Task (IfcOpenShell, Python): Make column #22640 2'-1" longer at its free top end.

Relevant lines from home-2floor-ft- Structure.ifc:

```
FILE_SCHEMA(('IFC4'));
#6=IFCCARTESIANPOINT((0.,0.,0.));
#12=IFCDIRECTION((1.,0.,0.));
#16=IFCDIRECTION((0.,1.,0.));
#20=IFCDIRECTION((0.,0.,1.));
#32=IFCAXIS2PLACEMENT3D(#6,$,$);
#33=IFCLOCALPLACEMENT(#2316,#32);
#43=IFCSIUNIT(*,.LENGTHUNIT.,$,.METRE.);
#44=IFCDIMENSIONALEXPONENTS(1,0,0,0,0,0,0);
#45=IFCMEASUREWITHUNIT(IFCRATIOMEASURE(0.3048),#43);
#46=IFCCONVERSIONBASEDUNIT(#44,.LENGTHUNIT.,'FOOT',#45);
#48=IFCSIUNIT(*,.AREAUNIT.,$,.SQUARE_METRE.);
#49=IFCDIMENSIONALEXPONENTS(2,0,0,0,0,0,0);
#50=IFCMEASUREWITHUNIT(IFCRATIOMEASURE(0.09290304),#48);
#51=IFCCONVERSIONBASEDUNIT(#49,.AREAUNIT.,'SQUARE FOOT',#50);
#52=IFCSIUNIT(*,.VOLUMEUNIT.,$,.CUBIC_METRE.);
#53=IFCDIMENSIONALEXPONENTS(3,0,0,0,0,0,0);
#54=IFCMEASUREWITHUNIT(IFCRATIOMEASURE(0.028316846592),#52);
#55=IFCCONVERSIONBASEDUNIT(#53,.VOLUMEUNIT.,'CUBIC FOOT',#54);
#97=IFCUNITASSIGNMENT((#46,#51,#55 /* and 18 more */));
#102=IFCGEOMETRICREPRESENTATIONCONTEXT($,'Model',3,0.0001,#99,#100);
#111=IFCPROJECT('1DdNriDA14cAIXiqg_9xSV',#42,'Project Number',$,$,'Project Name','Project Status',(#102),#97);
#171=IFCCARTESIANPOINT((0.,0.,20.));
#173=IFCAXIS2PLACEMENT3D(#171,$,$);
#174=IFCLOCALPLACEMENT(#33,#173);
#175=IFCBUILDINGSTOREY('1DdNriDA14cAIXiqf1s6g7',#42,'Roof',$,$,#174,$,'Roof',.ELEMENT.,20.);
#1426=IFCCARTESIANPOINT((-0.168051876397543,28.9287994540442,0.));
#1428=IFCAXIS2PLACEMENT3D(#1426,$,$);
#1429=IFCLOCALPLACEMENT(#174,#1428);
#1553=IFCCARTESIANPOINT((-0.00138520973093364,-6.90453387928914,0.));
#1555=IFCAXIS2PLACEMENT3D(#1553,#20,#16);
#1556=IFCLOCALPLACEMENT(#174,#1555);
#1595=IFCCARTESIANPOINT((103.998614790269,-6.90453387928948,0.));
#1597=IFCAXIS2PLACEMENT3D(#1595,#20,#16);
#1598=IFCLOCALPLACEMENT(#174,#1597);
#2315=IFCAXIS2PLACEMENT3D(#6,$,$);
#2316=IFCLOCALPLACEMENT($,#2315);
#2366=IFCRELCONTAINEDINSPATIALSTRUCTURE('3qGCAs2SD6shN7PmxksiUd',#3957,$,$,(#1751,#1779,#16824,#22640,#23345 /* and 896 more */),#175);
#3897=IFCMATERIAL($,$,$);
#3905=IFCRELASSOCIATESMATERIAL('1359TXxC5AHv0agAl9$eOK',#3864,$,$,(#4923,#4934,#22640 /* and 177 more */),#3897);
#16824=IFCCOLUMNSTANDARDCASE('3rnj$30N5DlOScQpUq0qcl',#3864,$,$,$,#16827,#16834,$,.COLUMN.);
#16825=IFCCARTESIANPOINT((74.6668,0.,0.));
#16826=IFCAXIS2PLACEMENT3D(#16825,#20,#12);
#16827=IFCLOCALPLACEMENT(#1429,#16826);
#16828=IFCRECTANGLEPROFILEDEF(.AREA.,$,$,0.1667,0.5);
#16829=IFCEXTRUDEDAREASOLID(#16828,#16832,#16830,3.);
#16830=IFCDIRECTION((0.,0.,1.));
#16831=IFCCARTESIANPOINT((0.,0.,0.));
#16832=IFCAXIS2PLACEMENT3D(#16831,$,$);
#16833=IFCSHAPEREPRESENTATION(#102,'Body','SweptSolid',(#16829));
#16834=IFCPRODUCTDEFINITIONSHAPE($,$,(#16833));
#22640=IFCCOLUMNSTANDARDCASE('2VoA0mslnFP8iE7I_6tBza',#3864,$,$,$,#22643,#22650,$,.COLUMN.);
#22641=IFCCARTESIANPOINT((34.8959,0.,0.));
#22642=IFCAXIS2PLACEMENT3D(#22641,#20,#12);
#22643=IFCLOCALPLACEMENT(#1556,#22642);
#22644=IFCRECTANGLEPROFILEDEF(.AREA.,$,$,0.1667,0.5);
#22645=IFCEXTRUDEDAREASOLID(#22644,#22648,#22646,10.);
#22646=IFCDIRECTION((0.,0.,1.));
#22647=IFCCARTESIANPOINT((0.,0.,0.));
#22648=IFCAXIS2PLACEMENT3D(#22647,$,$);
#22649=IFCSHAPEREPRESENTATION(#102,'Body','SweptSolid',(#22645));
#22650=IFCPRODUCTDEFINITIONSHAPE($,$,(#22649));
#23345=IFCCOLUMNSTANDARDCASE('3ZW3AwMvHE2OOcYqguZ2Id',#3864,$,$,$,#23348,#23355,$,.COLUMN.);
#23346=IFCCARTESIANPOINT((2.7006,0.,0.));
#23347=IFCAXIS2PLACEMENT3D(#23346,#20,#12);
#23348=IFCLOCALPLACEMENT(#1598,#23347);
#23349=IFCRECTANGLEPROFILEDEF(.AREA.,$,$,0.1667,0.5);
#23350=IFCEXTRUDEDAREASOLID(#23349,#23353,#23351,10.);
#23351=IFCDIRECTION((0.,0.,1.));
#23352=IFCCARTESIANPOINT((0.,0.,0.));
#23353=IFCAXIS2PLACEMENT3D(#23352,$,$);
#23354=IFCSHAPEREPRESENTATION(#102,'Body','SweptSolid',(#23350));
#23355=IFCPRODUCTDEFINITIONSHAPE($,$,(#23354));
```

```python
import ifcopenshell
import ifcopenshell.util.unit

model = ifcopenshell.open("home-2floor-ft- Structure.ifc")
unit_scale = ifcopenshell.util.unit.calculate_unit_scale(model)

member = model.by_guid("2VoA0mslnFP8iE7I_6tBza")
change = 25 * 0.0254 / unit_scale

# The extrusion runs towards the end named, so only its depth changes.
body = next(r for r in member.Representation.Representations if r.RepresentationIdentifier == "Body")
solid = body.Items[0]
old_length = solid.Depth
solid.Depth += change

print(f"length {old_length:g} -> {solid.Depth:g}")

model.write("home-2floor-ft- Structure_v2.ifc")
```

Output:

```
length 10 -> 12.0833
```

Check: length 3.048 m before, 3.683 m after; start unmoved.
